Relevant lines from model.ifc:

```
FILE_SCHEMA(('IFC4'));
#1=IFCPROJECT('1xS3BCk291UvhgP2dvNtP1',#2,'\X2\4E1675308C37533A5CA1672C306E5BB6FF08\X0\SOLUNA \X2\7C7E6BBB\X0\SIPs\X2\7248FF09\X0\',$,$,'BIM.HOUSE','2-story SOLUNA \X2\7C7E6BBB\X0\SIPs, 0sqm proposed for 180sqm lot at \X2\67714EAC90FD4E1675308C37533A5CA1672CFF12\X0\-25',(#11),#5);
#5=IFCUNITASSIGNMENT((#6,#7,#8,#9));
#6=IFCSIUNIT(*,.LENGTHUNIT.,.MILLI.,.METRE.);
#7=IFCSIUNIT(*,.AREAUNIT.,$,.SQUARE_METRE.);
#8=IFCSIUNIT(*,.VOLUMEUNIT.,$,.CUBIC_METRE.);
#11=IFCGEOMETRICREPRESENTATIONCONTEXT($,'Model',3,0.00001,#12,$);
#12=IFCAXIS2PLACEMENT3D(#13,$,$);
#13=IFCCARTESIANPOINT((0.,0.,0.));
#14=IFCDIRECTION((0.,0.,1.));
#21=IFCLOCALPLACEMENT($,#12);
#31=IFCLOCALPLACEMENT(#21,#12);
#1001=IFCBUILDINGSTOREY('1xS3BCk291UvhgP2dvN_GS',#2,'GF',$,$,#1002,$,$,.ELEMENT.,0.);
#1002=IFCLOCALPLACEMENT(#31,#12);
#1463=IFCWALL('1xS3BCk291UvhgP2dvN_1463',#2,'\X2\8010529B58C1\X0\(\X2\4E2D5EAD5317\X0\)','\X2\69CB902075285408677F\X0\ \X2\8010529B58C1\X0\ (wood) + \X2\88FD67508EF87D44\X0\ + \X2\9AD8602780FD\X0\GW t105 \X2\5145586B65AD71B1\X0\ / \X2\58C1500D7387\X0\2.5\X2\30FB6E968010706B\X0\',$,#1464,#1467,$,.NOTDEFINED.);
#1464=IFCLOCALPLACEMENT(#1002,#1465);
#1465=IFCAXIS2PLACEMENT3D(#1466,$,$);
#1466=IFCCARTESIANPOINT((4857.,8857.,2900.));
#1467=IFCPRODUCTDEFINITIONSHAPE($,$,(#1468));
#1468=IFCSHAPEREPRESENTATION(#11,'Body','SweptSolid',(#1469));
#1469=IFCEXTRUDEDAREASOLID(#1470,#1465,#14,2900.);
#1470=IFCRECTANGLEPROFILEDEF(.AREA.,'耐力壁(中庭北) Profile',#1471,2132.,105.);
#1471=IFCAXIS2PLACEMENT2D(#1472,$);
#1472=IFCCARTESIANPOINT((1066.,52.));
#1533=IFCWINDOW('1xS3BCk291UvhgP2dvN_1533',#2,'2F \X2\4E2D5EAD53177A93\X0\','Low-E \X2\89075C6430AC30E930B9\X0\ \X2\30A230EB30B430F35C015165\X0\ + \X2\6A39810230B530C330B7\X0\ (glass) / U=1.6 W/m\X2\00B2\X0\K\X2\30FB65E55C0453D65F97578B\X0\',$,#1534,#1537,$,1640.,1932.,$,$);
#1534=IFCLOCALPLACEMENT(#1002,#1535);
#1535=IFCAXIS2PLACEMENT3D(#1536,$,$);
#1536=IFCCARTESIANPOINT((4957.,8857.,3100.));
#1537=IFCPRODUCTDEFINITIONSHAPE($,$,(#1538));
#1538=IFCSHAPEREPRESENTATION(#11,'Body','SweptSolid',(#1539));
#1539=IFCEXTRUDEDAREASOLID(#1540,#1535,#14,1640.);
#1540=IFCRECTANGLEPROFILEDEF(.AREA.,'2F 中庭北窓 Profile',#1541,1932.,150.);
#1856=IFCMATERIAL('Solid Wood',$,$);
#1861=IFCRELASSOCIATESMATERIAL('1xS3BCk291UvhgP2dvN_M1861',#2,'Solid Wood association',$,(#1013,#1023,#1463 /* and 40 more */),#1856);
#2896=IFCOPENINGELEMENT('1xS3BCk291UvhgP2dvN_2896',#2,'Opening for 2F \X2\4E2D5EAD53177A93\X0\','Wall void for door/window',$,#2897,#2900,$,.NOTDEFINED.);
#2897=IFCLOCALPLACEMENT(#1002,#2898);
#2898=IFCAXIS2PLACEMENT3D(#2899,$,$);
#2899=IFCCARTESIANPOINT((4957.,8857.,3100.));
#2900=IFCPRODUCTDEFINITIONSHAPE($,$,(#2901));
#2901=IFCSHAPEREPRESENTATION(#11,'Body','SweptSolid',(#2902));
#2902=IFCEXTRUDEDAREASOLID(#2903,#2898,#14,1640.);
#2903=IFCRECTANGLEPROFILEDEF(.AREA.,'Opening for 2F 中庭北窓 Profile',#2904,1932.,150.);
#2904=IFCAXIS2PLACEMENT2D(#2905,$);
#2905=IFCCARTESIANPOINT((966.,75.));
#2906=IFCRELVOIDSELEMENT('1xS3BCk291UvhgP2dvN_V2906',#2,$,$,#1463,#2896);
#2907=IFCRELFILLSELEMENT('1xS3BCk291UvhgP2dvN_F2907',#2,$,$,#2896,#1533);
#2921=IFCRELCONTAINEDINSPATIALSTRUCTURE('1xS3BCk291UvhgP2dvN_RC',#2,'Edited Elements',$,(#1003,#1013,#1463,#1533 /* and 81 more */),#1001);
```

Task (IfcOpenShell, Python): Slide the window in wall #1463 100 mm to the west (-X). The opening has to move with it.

```python
import ifcopenshell
import ifcopenshell.api.geometry
import ifcopenshell.util.placement
import ifcopenshell.util.unit

model = ifcopenshell.open("model.ifc")
unit_scale = ifcopenshell.util.unit.calculate_unit_scale(model)

window = model.by_guid("1xS3BCk291UvhgP2dvN_1533")
opening = window.FillsVoids[0].RelatingOpeningElement
wall = opening.VoidsElements[0].RelatingBuildingElement

wall_matrix = ifcopenshell.util.placement.get_local_placement(wall.ObjectPlacement)
shift = wall_matrix[:3, 0] * -0.1 / unit_scale
before = ifcopenshell.util.placement.get_local_placement(window.ObjectPlacement)[:3, 3].copy()

# The window is not placed relative to its opening, so move both.
for product in (opening, window):
    matrix = ifcopenshell.util.placement.get_local_placement(product.ObjectPlacement)
    matrix[:3, 3] += shift
    ifcopenshell.api.geometry.edit_object_placement(model, product=product, matrix=matrix, is_si=False)

after = ifcopenshell.util.placement.get_local_placement(window.ObjectPlacement)[:3, 3]
print("window moved by", (after - before).round(3) + 0.0)

model.write("model_updated.ifc")
```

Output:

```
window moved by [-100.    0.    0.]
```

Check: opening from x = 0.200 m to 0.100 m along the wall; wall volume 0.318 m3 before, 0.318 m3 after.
